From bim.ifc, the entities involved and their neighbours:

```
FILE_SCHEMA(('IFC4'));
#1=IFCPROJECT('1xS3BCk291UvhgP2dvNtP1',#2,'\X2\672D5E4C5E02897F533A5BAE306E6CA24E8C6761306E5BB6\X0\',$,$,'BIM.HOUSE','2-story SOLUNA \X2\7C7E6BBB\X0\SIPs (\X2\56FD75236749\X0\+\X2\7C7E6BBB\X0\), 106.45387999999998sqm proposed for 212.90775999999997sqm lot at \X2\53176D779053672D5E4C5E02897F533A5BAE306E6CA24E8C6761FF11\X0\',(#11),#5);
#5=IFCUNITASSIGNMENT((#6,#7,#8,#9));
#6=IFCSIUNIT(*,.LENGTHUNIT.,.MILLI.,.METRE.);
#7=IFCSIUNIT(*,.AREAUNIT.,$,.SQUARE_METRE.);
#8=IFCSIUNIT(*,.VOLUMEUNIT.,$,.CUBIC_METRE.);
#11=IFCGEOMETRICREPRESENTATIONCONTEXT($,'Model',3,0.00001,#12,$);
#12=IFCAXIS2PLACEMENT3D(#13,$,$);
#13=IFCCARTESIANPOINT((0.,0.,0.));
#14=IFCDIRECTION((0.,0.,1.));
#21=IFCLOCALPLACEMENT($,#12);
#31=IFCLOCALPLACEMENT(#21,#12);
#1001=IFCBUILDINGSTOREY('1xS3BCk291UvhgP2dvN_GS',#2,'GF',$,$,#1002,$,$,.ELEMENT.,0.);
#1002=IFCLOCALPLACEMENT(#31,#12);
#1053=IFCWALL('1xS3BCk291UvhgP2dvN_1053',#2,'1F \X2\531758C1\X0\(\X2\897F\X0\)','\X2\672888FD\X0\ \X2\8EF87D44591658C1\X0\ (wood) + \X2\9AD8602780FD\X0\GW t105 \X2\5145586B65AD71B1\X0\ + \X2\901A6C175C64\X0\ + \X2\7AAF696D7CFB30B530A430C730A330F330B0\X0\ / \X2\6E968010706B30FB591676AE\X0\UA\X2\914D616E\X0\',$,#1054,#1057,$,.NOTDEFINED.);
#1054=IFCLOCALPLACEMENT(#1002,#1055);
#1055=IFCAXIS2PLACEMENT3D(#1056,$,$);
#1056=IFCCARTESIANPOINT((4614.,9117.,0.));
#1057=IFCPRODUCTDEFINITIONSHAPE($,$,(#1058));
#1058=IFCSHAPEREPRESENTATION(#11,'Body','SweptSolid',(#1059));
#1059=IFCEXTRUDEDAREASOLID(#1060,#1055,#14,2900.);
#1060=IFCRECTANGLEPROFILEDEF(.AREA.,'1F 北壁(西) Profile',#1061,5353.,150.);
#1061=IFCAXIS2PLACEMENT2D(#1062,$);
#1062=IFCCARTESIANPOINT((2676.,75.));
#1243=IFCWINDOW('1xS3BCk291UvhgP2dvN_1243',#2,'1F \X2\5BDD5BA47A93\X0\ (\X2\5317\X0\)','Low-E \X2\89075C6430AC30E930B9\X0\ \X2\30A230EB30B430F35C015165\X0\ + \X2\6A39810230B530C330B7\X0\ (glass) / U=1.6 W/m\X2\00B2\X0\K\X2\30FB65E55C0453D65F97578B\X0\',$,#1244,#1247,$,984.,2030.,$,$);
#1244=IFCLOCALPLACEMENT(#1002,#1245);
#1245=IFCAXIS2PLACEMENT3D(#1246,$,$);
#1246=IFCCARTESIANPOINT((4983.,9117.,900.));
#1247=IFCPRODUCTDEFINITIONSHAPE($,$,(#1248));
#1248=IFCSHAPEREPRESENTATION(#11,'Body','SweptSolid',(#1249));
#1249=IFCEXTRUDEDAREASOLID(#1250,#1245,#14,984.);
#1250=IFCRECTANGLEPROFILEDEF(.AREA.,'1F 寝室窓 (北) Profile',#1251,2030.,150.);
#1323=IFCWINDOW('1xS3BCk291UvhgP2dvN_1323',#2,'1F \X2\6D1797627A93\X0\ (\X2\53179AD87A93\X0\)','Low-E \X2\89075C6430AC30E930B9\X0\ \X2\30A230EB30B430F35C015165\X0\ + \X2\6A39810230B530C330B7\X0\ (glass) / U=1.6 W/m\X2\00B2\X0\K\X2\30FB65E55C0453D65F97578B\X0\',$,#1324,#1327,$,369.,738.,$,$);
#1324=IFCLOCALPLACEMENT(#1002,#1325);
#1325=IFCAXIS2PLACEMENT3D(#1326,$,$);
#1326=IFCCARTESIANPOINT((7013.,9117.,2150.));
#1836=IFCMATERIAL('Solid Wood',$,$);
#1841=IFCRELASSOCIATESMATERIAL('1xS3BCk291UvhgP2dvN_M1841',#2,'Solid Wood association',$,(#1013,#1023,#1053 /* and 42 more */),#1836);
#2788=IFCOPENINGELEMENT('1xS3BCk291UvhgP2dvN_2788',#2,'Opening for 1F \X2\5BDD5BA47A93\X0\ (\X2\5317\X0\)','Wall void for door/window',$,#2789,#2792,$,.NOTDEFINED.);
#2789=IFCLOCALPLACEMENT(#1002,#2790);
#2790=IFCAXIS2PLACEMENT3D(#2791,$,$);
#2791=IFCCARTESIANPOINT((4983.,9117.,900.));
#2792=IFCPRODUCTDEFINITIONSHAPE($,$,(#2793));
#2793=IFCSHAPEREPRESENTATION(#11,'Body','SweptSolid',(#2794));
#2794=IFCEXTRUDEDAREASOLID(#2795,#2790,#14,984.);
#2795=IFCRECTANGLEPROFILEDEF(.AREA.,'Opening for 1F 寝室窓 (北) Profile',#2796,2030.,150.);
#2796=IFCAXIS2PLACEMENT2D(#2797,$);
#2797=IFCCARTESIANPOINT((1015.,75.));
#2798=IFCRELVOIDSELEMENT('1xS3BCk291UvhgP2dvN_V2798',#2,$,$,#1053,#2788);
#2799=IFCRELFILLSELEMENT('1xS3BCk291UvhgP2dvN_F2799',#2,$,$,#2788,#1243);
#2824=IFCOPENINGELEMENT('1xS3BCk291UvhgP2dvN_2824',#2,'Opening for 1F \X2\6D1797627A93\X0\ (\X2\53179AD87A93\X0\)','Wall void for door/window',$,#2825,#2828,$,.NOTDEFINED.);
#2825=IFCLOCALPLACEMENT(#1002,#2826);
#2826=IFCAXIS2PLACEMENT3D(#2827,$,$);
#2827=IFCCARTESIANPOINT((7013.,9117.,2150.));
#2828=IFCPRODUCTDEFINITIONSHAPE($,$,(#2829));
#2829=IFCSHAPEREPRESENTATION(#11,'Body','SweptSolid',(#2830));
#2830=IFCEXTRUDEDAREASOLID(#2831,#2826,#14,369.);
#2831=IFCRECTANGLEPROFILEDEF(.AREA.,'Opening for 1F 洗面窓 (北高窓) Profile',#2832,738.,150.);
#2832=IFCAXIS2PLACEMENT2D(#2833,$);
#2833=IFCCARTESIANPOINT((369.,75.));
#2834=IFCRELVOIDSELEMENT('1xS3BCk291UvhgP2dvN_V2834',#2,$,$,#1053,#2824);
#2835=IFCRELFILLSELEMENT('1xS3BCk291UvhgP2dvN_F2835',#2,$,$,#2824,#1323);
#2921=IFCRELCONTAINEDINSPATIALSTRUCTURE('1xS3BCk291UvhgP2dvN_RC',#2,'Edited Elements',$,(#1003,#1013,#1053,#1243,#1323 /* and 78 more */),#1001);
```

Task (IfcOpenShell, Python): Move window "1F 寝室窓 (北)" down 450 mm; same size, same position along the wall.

```python
import numpy as np
import ifcopenshell
import ifcopenshell.api.geometry
import ifcopenshell.util.placement
import ifcopenshell.util.unit

model = ifcopenshell.open("bim.ifc")
unit_scale = ifcopenshell.util.unit.calculate_unit_scale(model)

window = model.by_guid("1xS3BCk291UvhgP2dvN_1243")
opening = window.FillsVoids[0].RelatingOpeningElement
dz = -0.45 / unit_scale

shift = np.array([0.0, 0.0, dz])
# The window is not placed relative to its opening, so move both.
for product in (opening, window):
    matrix = ifcopenshell.util.placement.get_local_placement(product.ObjectPlacement)
    matrix[:3, 3] += shift
    ifcopenshell.api.geometry.edit_object_placement(model, product=product, matrix=matrix, is_si=False)

print(f"moved by {dz * unit_scale:+.3f} m")

model.write("bim_rev.ifc")
```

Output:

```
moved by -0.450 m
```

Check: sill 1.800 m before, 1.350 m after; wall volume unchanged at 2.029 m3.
